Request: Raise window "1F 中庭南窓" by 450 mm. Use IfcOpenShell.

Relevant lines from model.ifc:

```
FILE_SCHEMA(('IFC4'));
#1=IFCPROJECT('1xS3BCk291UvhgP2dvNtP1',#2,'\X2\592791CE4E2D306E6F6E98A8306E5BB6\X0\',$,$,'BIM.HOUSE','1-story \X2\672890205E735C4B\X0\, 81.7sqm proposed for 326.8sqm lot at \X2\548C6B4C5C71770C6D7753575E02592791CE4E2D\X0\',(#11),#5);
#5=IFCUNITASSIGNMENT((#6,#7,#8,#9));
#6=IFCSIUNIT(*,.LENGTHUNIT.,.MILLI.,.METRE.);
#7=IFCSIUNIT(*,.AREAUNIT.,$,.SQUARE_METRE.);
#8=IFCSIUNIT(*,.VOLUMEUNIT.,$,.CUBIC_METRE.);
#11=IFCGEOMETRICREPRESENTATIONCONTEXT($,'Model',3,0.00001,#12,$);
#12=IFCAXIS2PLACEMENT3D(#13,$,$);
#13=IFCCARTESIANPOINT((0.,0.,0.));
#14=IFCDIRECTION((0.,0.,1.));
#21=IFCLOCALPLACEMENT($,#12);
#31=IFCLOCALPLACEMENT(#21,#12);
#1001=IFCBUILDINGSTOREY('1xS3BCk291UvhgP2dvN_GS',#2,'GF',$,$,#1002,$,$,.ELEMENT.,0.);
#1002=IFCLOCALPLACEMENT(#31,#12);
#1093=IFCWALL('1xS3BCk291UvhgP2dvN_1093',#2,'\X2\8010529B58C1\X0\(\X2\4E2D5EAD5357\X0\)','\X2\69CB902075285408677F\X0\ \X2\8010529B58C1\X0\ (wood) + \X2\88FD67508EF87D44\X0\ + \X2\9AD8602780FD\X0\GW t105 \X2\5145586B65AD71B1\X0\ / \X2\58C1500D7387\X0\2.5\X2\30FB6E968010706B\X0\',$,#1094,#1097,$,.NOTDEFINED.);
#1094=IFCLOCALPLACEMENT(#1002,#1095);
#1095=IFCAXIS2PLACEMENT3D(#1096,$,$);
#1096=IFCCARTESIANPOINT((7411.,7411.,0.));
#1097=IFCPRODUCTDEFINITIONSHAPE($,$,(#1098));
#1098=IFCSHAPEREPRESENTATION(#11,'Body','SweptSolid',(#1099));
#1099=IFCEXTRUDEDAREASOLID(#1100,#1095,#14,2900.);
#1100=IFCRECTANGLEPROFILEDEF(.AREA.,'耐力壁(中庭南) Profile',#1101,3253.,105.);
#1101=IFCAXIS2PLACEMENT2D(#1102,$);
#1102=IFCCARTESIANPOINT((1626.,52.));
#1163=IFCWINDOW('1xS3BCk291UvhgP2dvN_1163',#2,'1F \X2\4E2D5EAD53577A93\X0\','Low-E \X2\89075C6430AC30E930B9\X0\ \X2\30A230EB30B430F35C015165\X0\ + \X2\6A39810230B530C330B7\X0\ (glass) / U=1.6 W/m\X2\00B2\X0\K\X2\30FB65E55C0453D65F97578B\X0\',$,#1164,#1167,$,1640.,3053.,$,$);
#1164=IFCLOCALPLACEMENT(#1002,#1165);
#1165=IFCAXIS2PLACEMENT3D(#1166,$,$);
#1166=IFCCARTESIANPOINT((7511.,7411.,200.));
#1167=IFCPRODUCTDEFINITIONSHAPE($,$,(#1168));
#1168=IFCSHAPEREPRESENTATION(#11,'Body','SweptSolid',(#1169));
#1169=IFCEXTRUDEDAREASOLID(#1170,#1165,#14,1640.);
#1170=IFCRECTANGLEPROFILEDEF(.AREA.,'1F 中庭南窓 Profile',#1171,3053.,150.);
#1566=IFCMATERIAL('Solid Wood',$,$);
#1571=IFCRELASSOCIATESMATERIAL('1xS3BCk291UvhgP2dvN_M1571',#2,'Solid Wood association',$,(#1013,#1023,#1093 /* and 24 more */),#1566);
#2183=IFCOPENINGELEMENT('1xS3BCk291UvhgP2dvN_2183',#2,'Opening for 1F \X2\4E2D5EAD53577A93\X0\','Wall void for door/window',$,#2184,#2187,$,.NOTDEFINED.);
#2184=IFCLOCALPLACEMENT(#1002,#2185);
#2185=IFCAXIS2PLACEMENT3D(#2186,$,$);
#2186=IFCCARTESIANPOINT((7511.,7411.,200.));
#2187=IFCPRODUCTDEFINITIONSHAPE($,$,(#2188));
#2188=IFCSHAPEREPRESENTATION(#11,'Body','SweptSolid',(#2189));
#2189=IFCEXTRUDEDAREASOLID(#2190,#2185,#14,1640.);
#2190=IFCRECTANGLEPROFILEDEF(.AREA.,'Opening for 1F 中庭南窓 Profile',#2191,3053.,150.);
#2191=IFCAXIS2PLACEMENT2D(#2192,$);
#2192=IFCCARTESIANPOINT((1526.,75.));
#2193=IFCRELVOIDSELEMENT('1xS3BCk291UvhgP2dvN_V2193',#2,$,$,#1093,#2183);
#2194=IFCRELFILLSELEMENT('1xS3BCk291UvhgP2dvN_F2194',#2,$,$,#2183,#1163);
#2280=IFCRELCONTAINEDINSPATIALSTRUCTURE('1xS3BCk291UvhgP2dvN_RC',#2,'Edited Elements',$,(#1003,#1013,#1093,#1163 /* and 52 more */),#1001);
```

```python
import numpy as np
import ifcopenshell
import ifcopenshell.api.geometry
import ifcopenshell.util.placement
import ifcopenshell.util.unit

model = ifcopenshell.open("model.ifc")
unit_scale = ifcopenshell.util.unit.calculate_unit_scale(model)

window = model.by_guid("1xS3BCk291UvhgP2dvN_1163")
opening = window.FillsVoids[0].RelatingOpeningElement
dz = 450.0

shift = np.array([0.0, 0.0, dz])
# The window is not placed relative to its opening, so move both.
for product in (opening, window):
    matrix = ifcopenshell.util.placement.get_local_placement(product.ObjectPlacement)
    matrix[:3, 3] += shift
    ifcopenshell.api.geometry.edit_object_placement(model, product=product, matrix=matrix, is_si=False)

print(f"moved by {dz * unit_scale:+.3f} m")

model.write("model_updated.ifc")
```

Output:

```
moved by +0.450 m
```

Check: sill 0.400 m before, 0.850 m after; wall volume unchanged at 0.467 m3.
